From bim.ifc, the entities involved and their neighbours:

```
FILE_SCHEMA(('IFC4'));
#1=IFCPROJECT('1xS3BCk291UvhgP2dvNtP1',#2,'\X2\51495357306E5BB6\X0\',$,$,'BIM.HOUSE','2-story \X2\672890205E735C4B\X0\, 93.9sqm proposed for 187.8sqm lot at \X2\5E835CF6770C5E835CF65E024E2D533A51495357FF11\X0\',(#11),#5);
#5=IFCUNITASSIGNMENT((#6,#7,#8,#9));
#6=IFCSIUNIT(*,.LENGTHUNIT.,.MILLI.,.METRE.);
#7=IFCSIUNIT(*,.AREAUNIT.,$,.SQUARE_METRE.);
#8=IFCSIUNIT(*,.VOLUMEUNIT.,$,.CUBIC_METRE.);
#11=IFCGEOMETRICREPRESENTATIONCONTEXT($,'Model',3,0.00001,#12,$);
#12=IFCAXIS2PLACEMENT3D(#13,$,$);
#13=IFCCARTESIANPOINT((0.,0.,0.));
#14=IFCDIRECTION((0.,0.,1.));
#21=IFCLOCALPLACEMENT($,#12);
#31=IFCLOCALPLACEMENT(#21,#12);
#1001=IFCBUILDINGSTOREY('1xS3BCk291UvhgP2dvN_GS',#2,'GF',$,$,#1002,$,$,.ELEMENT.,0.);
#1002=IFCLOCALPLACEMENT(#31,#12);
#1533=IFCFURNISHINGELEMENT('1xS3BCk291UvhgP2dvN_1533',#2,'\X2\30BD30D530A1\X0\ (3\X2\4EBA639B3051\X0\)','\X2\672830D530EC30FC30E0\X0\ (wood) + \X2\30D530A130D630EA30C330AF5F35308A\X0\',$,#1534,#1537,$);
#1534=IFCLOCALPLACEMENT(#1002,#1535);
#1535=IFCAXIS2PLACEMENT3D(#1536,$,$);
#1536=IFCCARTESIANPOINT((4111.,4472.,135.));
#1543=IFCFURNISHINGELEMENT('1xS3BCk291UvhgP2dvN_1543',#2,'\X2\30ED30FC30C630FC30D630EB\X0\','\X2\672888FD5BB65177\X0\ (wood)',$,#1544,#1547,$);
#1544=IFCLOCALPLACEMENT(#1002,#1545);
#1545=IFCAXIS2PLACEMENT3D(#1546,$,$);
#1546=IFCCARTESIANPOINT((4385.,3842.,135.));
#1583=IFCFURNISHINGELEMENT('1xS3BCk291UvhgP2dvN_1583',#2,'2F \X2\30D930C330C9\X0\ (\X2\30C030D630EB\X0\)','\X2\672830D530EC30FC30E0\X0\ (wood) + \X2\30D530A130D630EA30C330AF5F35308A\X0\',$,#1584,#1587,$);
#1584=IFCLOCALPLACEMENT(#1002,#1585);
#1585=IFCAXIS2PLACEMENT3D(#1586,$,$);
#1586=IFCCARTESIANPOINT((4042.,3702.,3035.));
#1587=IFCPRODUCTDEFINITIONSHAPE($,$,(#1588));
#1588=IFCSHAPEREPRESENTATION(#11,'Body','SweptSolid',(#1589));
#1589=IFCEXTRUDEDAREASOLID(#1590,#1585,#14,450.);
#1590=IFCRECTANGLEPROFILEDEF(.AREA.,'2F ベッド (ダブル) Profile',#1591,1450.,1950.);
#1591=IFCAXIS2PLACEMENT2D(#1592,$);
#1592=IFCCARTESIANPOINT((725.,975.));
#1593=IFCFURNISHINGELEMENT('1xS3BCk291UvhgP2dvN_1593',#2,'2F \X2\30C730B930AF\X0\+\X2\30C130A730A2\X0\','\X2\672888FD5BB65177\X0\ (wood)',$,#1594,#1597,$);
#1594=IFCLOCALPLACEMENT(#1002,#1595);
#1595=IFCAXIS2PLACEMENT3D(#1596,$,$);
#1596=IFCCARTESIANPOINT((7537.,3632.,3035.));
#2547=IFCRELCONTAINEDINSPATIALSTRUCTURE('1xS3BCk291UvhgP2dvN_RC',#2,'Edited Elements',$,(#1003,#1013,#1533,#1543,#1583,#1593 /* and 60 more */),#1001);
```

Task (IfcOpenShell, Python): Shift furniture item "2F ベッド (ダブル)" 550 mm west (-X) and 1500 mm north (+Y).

```python
import ifcopenshell
import ifcopenshell.api.geometry
import ifcopenshell.util.placement
import ifcopenshell.util.unit

model = ifcopenshell.open("bim.ifc")
unit_scale = ifcopenshell.util.unit.calculate_unit_scale(model)

item = model.by_guid("1xS3BCk291UvhgP2dvN_1583")
matrix = ifcopenshell.util.placement.get_local_placement(item.ObjectPlacement)
matrix[0, 3] -= 0.55 / unit_scale
matrix[1, 3] += 1.5 / unit_scale
ifcopenshell.api.geometry.edit_object_placement(model, product=item, matrix=matrix, is_si=False)

print(ifcopenshell.util.placement.get_local_placement(item.ObjectPlacement).round(3) + 0.0)

model.write("bim-out.ifc")
```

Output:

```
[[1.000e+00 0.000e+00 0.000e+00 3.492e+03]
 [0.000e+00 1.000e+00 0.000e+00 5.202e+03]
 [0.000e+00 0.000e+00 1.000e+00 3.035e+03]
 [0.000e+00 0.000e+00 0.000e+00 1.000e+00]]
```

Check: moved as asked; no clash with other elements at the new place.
